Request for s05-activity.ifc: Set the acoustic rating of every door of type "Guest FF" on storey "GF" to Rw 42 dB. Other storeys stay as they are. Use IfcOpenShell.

First a look at what the model holds.

```python
import ifcopenshell
import ifcopenshell.util.element

model = ifcopenshell.open("s05-activity.ifc")
print(model.schema)
storey = next(s for s in model.by_type("IfcBuildingStorey") if s.Name == "GF")
doors = [e for e in ifcopenshell.util.element.get_decomposition(storey) if e.is_a("IfcDoor")]
seen = {}
for e in doors:
    element_type = ifcopenshell.util.element.get_type(e)
    key = (element_type.Name if element_type != e and element_type else None, ifcopenshell.util.element.get_pset(e, "Pset_DoorCommon", "AcousticRating"))
    seen[key] = seen.get(key, 0) + 1
for (name, value), count in sorted(seen.items(), key=str):
    print(count, "x", name, "|", value)
```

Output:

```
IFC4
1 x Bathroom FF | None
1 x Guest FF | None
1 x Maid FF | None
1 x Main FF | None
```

```python
import ifcopenshell
import ifcopenshell.api.pset
import ifcopenshell.util.element

model = ifcopenshell.open("s05-activity.ifc")

storey = next(s for s in model.by_type("IfcBuildingStorey") if s.Name == "GF")
doors = [e for e in ifcopenshell.util.element.get_decomposition(storey) if e.is_a("IfcDoor")]

count = 0
for e in doors:
    element_type = ifcopenshell.util.element.get_type(e)
    if element_type in (None, e) or element_type.Name != "Guest FF":
        continue
    # add_pset returns the element's existing set when there is one.
    pset = ifcopenshell.api.pset.add_pset(model, product=e, name="Pset_DoorCommon")
    ifcopenshell.api.pset.edit_pset(model, pset=pset, properties={"AcousticRating": "Rw 42 dB"})
    count += 1

print(count, "doors updated")

model.write("s05-activity-out.ifc")
```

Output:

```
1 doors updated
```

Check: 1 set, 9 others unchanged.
